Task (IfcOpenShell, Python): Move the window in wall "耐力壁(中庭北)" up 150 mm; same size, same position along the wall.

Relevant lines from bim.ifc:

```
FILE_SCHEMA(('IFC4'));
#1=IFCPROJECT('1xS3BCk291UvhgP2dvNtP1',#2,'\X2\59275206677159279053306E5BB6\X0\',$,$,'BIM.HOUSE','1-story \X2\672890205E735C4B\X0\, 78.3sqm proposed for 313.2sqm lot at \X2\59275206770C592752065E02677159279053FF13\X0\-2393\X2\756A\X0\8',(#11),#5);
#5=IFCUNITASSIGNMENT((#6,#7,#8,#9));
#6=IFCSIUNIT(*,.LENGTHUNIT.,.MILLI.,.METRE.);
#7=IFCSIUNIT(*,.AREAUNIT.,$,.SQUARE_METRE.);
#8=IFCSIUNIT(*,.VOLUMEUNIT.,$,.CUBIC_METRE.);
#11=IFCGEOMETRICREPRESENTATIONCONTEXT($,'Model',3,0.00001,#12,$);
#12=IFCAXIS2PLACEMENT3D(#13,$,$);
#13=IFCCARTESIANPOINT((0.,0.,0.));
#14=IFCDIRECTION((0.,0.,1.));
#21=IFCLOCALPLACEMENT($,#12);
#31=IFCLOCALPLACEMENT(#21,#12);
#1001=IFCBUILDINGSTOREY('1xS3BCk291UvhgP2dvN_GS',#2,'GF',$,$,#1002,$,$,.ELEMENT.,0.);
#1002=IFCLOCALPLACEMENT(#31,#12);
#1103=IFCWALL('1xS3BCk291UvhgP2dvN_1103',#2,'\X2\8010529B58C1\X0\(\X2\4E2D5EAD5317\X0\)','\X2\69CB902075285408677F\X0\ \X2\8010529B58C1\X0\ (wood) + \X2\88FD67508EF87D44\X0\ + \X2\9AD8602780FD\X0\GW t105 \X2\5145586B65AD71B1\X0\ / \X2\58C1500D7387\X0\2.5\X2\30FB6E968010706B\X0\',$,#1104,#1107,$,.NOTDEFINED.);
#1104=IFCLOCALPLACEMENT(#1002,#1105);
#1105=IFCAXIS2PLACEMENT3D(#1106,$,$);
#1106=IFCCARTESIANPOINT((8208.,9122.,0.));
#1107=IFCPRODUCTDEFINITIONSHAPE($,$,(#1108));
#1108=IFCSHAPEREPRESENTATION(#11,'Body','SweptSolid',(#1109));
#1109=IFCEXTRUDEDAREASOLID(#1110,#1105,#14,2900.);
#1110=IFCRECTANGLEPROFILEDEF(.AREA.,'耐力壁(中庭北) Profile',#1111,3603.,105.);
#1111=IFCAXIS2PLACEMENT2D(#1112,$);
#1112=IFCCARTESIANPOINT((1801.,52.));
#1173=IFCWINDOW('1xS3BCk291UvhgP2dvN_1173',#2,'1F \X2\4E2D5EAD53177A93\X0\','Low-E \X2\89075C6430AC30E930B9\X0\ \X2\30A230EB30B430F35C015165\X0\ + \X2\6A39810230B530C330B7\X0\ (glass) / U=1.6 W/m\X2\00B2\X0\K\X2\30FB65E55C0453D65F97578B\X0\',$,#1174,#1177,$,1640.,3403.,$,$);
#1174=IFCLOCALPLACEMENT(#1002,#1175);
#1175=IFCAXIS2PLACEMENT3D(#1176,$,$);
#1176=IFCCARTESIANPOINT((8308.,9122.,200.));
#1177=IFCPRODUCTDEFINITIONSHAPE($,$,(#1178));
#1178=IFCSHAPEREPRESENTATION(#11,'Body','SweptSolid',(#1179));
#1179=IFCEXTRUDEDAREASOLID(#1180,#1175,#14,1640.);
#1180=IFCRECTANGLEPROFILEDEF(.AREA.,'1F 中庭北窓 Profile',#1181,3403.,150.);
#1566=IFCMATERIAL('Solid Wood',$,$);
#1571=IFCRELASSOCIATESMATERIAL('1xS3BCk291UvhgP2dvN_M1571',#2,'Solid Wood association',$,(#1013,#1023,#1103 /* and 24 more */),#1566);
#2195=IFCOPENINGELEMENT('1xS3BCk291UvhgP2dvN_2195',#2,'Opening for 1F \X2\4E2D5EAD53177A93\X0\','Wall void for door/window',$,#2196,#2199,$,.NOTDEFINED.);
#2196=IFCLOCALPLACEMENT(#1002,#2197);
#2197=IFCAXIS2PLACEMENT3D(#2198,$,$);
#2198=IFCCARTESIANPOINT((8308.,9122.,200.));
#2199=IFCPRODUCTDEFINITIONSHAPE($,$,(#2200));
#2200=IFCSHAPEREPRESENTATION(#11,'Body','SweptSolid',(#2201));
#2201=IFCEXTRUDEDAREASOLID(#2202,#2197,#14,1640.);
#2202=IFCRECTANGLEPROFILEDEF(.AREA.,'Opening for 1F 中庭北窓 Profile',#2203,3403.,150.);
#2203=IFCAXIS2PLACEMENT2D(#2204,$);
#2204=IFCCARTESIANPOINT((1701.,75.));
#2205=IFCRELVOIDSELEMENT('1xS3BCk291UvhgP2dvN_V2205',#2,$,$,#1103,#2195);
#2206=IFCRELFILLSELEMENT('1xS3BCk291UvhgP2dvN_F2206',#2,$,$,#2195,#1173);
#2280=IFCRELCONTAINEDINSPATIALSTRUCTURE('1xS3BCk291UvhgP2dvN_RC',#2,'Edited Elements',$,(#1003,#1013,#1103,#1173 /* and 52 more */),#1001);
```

```python
import numpy as np
import ifcopenshell
import ifcopenshell.api.geometry
import ifcopenshell.util.placement
import ifcopenshell.util.unit

model = ifcopenshell.open("bim.ifc")
unit_scale = ifcopenshell.util.unit.calculate_unit_scale(model)

window = model.by_id(1173)
opening = window.FillsVoids[0].RelatingOpeningElement
dz = 150.0

shift = np.array([0.0, 0.0, dz])
# The window is not placed relative to its opening, so move both.
for product in (opening, window):
    matrix = ifcopenshell.util.placement.get_local_placement(product.ObjectPlacement)
    matrix[:3, 3] += shift
    ifcopenshell.api.geometry.edit_object_placement(model, product=product, matrix=matrix, is_si=False)

print(f"moved by {dz * unit_scale:+.3f} m")

model.write("bim_v2.ifc")
```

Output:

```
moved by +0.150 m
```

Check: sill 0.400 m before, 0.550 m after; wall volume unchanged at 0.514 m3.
